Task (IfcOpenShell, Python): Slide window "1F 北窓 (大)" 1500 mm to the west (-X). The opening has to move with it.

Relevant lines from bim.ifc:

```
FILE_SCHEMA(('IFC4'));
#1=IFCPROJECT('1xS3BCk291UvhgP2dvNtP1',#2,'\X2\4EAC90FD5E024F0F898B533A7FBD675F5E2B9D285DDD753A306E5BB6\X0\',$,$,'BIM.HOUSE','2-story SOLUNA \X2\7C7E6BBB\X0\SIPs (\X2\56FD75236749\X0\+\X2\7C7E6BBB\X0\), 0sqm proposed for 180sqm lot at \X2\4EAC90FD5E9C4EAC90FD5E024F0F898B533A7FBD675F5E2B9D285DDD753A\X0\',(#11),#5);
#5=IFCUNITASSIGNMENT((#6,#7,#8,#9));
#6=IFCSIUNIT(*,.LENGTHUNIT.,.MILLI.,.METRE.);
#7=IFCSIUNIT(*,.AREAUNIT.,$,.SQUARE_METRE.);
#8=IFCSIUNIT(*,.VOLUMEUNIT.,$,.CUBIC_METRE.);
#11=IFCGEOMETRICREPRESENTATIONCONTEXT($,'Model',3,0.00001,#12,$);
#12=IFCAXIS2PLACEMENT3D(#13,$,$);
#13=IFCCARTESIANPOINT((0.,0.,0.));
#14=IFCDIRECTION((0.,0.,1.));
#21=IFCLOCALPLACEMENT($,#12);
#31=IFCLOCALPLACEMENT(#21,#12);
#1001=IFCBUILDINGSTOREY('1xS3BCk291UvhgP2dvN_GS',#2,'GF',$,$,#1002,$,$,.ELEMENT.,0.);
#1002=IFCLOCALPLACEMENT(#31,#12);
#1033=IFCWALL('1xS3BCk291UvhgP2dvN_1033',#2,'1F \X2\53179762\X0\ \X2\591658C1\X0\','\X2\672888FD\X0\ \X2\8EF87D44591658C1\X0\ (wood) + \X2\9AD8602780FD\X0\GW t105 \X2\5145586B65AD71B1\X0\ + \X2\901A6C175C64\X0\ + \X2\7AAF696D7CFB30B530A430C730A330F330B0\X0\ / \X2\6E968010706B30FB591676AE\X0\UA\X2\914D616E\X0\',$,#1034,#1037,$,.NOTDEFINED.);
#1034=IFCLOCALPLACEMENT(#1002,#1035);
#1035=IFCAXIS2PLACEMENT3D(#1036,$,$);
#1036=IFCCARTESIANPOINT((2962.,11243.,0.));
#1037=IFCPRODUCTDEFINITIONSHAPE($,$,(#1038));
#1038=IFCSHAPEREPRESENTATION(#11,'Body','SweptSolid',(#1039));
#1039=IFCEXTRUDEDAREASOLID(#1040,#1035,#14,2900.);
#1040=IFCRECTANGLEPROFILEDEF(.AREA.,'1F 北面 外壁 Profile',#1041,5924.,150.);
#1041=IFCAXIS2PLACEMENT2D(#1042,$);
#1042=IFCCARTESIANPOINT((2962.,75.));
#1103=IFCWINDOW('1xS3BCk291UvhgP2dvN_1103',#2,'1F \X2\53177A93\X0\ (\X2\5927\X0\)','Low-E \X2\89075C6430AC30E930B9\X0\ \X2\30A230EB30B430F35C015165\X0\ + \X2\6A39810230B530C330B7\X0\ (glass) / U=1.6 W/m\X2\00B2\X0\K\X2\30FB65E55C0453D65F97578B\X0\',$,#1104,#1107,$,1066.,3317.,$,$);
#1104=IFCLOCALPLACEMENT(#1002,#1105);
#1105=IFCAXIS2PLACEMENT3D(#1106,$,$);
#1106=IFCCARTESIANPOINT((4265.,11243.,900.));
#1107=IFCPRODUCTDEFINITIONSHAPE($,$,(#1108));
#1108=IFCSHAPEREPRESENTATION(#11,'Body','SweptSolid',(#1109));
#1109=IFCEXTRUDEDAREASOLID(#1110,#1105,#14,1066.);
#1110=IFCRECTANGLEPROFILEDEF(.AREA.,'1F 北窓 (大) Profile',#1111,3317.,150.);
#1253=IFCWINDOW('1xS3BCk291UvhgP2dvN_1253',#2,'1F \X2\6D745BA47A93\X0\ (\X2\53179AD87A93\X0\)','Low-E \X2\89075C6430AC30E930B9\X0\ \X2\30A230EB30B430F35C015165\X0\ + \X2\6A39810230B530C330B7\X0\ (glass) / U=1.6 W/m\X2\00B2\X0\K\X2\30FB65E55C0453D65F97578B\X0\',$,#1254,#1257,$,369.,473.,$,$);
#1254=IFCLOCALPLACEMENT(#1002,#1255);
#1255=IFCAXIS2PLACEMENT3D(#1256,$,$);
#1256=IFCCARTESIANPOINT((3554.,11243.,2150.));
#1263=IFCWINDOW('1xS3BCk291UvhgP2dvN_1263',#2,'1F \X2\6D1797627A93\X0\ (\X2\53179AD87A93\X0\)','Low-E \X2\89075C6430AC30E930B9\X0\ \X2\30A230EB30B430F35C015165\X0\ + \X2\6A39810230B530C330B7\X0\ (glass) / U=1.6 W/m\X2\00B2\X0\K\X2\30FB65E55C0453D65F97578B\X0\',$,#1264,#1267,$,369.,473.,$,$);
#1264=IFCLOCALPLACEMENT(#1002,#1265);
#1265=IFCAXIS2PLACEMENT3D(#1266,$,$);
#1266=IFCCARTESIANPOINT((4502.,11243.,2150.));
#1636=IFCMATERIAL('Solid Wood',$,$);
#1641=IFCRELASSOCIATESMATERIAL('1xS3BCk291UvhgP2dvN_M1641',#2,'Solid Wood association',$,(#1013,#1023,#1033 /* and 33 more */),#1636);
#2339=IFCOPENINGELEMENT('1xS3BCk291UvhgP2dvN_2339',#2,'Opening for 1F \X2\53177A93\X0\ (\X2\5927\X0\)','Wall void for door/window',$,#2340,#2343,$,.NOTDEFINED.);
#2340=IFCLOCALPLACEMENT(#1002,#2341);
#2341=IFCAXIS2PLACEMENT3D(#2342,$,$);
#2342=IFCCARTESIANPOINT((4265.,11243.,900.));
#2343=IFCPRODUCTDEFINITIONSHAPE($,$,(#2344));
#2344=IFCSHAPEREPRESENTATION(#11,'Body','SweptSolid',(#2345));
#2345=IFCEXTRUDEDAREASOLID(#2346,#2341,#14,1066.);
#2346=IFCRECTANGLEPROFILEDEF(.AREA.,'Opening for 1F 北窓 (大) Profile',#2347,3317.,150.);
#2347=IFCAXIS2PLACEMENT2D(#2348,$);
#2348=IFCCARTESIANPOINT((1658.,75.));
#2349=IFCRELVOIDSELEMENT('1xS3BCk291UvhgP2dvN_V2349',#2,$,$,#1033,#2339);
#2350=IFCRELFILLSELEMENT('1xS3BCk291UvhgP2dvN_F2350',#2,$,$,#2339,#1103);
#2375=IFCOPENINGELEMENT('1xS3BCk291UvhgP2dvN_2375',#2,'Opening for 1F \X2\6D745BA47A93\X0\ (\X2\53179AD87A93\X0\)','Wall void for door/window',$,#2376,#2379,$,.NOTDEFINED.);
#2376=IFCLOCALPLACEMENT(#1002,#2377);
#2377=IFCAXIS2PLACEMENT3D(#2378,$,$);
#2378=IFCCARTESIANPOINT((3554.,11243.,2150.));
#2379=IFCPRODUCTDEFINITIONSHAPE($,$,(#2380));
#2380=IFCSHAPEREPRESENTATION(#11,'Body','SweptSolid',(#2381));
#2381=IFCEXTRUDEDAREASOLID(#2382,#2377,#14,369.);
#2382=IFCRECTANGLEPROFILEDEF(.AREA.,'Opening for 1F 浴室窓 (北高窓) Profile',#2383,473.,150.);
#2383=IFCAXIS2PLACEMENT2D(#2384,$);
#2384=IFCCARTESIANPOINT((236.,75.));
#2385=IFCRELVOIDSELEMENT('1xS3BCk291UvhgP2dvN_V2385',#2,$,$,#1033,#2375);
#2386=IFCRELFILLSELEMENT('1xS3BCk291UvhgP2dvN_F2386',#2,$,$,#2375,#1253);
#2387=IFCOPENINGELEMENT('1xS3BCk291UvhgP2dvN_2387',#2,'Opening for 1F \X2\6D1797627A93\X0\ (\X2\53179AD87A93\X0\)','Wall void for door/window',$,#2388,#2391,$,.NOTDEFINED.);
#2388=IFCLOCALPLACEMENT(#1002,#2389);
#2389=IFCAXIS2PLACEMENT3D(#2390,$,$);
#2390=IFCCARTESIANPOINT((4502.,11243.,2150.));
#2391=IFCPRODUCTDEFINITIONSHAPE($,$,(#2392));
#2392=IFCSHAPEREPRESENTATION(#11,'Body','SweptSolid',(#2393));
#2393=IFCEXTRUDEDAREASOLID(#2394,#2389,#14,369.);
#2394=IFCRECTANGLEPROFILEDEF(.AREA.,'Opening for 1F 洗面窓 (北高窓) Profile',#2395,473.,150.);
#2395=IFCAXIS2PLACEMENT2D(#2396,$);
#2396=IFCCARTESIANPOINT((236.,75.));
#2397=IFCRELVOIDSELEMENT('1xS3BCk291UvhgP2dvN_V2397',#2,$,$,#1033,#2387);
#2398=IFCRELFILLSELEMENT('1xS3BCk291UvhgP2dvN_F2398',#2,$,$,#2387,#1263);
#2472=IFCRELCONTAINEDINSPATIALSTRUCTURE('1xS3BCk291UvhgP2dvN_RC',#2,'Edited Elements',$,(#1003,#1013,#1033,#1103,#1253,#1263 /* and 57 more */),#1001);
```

```python
import ifcopenshell
import ifcopenshell.api.geometry
import ifcopenshell.util.placement
import ifcopenshell.util.unit

model = ifcopenshell.open("bim.ifc")
unit_scale = ifcopenshell.util.unit.calculate_unit_scale(model)

window = model.by_guid("1xS3BCk291UvhgP2dvN_1103")
opening = window.FillsVoids[0].RelatingOpeningElement
wall = opening.VoidsElements[0].RelatingBuildingElement

wall_matrix = ifcopenshell.util.placement.get_local_placement(wall.ObjectPlacement)
shift = wall_matrix[:3, 0] * -1.5 / unit_scale
before = ifcopenshell.util.placement.get_local_placement(window.ObjectPlacement)[:3, 3].copy()

# The window is not placed relative to its opening, so move both.
for product in (opening, window):
    matrix = ifcopenshell.util.placement.get_local_placement(product.ObjectPlacement)
    matrix[:3, 3] += shift
    ifcopenshell.api.geometry.edit_object_placement(model, product=product, matrix=matrix, is_si=False)

after = ifcopenshell.util.placement.get_local_placement(window.ObjectPlacement)[:3, 3]
print("window moved by", (after - before).round(3) + 0.0)

model.write("bim_updated.ifc")
```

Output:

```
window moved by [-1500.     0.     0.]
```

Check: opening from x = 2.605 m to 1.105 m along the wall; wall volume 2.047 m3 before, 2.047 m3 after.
